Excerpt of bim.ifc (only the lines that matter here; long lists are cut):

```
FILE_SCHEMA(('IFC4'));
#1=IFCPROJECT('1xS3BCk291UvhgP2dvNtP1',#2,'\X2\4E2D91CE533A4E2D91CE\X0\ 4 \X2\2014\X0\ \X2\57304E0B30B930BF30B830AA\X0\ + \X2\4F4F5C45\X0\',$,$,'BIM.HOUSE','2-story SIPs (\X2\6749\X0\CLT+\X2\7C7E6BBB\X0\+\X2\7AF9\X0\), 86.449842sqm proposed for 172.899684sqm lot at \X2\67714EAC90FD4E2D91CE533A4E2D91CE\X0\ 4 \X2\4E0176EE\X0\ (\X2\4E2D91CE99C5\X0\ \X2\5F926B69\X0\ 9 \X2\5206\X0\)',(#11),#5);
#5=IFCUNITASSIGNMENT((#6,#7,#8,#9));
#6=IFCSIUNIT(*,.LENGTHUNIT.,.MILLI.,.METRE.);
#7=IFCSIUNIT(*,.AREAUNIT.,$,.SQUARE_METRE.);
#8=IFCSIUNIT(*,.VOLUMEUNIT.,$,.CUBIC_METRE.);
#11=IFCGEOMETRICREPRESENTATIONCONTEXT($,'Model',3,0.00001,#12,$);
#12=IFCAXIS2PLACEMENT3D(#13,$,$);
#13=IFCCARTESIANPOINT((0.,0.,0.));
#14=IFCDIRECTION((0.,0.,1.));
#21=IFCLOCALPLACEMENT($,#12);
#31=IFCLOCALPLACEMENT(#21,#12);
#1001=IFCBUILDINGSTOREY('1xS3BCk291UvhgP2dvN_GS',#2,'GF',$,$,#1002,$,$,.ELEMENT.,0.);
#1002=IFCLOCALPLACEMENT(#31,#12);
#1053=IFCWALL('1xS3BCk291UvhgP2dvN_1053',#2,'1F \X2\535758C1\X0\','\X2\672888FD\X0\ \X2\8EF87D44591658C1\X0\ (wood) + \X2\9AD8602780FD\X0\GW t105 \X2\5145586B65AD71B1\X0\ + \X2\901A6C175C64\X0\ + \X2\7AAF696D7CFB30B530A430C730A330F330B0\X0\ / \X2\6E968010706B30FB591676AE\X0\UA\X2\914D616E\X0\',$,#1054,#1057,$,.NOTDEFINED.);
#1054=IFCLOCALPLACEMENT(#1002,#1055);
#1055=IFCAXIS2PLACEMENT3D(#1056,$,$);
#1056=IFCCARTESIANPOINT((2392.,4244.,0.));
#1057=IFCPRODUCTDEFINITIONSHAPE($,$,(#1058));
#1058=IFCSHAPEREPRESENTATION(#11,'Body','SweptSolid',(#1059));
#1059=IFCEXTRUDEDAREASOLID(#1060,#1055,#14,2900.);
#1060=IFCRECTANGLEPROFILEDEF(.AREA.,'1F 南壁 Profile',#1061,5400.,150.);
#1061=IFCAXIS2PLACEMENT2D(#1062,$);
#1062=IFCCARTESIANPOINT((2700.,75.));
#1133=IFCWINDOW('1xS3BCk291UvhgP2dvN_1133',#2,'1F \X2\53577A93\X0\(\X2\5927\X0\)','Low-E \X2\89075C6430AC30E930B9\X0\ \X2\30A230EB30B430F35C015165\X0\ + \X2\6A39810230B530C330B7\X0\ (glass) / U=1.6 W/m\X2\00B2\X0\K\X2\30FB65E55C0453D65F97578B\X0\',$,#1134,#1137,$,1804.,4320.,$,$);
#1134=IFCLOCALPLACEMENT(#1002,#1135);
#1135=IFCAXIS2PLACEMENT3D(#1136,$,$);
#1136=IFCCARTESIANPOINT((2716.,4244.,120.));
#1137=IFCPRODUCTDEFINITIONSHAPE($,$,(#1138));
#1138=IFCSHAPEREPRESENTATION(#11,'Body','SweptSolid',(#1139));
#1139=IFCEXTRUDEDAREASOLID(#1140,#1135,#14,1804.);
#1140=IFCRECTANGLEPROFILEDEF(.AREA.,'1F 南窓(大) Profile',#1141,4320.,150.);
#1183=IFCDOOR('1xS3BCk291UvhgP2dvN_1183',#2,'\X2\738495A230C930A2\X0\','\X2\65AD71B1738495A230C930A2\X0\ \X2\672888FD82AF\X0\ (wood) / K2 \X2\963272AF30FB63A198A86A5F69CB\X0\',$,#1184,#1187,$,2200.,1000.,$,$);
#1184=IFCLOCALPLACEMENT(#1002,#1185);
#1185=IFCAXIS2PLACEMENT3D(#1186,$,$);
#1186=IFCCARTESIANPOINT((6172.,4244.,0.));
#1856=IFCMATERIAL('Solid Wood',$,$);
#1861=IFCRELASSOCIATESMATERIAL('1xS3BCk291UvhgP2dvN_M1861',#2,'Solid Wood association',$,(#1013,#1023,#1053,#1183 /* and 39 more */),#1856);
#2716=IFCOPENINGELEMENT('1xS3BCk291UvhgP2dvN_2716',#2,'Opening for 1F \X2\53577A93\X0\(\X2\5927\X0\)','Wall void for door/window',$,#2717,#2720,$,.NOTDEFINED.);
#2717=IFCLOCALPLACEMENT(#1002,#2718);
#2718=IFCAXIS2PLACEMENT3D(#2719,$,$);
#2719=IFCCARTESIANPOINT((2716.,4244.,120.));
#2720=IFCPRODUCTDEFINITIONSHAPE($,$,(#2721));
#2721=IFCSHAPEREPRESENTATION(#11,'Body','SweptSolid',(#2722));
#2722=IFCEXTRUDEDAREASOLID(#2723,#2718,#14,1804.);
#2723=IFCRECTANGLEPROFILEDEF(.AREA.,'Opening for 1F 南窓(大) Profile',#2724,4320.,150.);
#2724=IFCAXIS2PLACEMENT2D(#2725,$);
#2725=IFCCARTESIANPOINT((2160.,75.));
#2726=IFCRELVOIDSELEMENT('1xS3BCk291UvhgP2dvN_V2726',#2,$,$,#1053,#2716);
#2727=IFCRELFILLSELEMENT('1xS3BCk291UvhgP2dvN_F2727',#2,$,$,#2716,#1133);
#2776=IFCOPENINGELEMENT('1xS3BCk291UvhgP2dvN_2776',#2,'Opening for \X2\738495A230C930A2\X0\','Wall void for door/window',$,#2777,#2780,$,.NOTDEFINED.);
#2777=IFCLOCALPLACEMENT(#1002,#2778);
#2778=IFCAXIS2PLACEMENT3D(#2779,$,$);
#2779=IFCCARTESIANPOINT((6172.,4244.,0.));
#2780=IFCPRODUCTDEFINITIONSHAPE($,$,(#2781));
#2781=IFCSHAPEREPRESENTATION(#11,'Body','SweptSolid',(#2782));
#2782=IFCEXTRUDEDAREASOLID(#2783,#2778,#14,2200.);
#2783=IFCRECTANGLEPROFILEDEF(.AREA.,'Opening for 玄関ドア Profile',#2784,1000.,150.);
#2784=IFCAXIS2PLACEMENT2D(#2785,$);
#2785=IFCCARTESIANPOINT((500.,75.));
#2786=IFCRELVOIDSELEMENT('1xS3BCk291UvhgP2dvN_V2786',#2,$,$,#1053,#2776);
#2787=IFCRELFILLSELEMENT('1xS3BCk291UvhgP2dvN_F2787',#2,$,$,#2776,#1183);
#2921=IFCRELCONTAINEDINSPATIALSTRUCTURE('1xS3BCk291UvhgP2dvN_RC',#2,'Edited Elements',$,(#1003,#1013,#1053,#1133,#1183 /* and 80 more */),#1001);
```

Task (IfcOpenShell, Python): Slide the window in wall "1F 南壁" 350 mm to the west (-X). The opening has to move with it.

```python
import ifcopenshell
import ifcopenshell.api.geometry
import ifcopenshell.util.placement
import ifcopenshell.util.unit

model = ifcopenshell.open("bim.ifc")
unit_scale = ifcopenshell.util.unit.calculate_unit_scale(model)

window = model.by_guid("1xS3BCk291UvhgP2dvN_1133")
opening = window.FillsVoids[0].RelatingOpeningElement
wall = opening.VoidsElements[0].RelatingBuildingElement

wall_matrix = ifcopenshell.util.placement.get_local_placement(wall.ObjectPlacement)
shift = wall_matrix[:3, 0] * -0.35 / unit_scale
before = ifcopenshell.util.placement.get_local_placement(window.ObjectPlacement)[:3, 3].copy()

# The window is not placed relative to its opening, so move both.
for product in (opening, window):
    matrix = ifcopenshell.util.placement.get_local_placement(product.ObjectPlacement)
    matrix[:3, 3] += shift
    ifcopenshell.api.geometry.edit_object_placement(model, product=product, matrix=matrix, is_si=False)

after = ifcopenshell.util.placement.get_local_placement(window.ObjectPlacement)[:3, 3]
print("window moved by", (after - before).round(3) + 0.0)

model.write("bim_v2.ifc")
```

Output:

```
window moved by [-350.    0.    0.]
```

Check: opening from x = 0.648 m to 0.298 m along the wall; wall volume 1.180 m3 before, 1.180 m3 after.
